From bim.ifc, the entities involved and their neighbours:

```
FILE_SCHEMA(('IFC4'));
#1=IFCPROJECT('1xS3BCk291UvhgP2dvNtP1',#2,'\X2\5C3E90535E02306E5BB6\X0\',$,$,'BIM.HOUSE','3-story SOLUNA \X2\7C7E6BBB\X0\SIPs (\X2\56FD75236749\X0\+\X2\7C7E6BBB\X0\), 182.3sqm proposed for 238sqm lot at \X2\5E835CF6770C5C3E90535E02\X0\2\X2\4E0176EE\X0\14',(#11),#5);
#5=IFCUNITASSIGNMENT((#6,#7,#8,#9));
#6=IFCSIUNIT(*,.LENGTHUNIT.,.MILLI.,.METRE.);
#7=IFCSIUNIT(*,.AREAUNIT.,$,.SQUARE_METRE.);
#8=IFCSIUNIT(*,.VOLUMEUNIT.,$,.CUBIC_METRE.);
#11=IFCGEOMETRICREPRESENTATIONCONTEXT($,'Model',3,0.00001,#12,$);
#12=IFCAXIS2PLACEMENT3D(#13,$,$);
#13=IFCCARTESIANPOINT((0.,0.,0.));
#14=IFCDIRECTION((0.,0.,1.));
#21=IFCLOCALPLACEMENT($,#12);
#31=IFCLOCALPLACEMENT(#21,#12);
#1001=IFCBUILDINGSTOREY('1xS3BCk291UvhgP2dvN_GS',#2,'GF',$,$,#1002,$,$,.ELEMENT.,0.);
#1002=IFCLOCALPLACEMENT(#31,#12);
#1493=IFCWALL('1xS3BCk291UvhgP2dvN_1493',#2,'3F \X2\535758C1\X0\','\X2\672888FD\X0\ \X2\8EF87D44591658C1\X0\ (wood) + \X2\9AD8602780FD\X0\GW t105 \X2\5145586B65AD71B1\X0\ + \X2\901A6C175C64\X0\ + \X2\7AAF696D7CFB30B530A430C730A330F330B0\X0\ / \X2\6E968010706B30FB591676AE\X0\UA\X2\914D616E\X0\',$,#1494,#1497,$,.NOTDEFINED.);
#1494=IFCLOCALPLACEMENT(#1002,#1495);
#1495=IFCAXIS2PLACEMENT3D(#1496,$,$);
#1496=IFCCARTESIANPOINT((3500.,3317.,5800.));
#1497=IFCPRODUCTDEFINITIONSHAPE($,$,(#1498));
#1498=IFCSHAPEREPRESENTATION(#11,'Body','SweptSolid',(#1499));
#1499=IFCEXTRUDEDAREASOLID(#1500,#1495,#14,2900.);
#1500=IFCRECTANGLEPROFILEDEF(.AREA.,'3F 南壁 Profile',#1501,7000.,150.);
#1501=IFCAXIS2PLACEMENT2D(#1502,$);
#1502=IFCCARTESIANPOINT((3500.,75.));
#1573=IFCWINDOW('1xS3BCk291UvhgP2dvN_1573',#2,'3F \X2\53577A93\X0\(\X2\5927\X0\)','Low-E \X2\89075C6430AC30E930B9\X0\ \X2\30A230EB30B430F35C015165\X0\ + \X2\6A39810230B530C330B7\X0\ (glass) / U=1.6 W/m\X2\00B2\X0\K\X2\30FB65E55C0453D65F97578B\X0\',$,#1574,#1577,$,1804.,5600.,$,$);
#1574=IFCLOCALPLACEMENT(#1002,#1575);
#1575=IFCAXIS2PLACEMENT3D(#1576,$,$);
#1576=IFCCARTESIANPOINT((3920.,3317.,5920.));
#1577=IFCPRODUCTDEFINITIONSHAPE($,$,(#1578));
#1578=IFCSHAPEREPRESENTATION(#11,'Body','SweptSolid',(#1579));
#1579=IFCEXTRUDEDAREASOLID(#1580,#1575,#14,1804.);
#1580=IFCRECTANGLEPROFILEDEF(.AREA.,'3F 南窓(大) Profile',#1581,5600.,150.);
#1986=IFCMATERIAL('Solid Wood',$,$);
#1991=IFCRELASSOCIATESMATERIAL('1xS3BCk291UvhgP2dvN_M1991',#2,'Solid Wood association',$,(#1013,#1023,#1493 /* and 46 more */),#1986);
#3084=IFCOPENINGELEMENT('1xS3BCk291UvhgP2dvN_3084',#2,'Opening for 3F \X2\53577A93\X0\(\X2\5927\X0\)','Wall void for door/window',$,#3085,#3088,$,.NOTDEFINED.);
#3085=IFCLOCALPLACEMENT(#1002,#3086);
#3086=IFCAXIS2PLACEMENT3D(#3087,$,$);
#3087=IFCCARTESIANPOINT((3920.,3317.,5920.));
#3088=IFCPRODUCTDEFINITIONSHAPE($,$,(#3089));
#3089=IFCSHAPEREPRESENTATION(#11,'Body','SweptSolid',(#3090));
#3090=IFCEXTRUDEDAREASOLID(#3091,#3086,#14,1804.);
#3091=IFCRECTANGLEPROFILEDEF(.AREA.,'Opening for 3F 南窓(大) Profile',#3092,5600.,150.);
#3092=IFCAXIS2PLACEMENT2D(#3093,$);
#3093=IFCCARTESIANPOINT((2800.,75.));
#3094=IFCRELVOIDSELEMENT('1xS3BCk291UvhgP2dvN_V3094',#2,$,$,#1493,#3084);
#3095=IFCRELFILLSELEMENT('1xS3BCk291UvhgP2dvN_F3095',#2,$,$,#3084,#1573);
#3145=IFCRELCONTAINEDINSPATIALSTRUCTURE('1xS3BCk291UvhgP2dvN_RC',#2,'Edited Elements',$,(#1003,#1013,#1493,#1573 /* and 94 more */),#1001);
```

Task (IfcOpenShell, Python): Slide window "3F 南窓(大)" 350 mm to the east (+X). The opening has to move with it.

```python
import ifcopenshell
import ifcopenshell.api.geometry
import ifcopenshell.util.placement

model = ifcopenshell.open("bim.ifc")

window = model.by_id(1573)
opening = window.FillsVoids[0].RelatingOpeningElement
wall = opening.VoidsElements[0].RelatingBuildingElement

wall_matrix = ifcopenshell.util.placement.get_local_placement(wall.ObjectPlacement)
shift = wall_matrix[:3, 0] * 350.0
before = ifcopenshell.util.placement.get_local_placement(window.ObjectPlacement)[:3, 3].copy()

# The window is not placed relative to its opening, so move both.
for product in (opening, window):
    matrix = ifcopenshell.util.placement.get_local_placement(product.ObjectPlacement)
    matrix[:3, 3] += shift
    ifcopenshell.api.geometry.edit_object_placement(model, product=product, matrix=matrix, is_si=False)

after = ifcopenshell.util.placement.get_local_placement(window.ObjectPlacement)[:3, 3]
print("window moved by", (after - before).round(3) + 0.0)

model.write("bim_edited.ifc")
```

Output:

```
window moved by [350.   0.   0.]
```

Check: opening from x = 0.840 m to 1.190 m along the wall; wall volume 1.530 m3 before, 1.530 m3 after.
